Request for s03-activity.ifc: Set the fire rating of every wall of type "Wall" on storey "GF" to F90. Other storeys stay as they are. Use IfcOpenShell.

First a look at what the model holds.

```python
import ifcopenshell
import ifcopenshell.util.element

model = ifcopenshell.open("s03-activity.ifc")
print(model.schema)
storey = next(s for s in model.by_type("IfcBuildingStorey") if s.Name == "GF")
walls = [e for e in ifcopenshell.util.element.get_decomposition(storey) if e.is_a("IfcWall")]
seen = {}
for e in walls:
    element_type = ifcopenshell.util.element.get_type(e)
    key = (element_type.Name if element_type != e and element_type else None, ifcopenshell.util.element.get_pset(e, "Pset_WallCommon", "FireRating"))
    seen[key] = seen.get(key, 0) + 1
for (name, value), count in sorted(seen.items(), key=str):
    print(count, "x", name, "|", value)
```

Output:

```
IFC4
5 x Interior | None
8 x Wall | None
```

```python
import ifcopenshell
import ifcopenshell.api.pset
import ifcopenshell.util.element

model = ifcopenshell.open("s03-activity.ifc")

storey = next(s for s in model.by_type("IfcBuildingStorey") if s.Name == "GF")
walls = [e for e in ifcopenshell.util.element.get_decomposition(storey) if e.is_a("IfcWall")]

count = 0
for e in walls:
    element_type = ifcopenshell.util.element.get_type(e)
    if element_type in (None, e) or element_type.Name != "Wall":
        continue
    # add_pset returns the element's existing set when there is one.
    pset = ifcopenshell.api.pset.add_pset(model, product=e, name="Pset_WallCommon")
    ifcopenshell.api.pset.edit_pset(model, pset=pset, properties={"FireRating": "F90"})
    count += 1

print(count, "walls updated")

model.write("s03-activity_edited.ifc")
```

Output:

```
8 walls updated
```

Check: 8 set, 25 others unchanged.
